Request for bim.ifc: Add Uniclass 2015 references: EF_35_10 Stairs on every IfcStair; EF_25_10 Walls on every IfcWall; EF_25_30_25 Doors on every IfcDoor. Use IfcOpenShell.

First a look at what the model holds.

```python
import ifcopenshell

model = ifcopenshell.open("bim.ifc")
print(model.schema)
print("classifications:", [c.Name for c in model.by_type("IfcClassification")])
for ifc_class in ("IfcDoor", "IfcRoof", "IfcStair", "IfcWall", "IfcWindow"):
    print(ifc_class, len(model.by_type(ifc_class)))
```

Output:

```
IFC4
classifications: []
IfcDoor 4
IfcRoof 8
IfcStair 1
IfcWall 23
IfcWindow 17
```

```python
import ifcopenshell
import ifcopenshell.api.classification

model = ifcopenshell.open("bim.ifc")

system = ifcopenshell.api.classification.add_classification(model, classification="Uniclass 2015")

codes = {
    "IfcStair": ("EF_35_10", "Stairs"),
    "IfcWall": ("EF_25_10", "Walls"),
    "IfcDoor": ("EF_25_30_25", "Doors"),
}
for ifc_class, (code, name) in codes.items():
    products = model.by_type(ifc_class)
    ifcopenshell.api.classification.add_reference(
        model, products=products, classification=system, identification=code, name=name
    )
    print(code, len(products))

model.write("bim_edited.ifc")
```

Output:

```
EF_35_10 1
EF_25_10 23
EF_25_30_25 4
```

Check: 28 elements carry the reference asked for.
